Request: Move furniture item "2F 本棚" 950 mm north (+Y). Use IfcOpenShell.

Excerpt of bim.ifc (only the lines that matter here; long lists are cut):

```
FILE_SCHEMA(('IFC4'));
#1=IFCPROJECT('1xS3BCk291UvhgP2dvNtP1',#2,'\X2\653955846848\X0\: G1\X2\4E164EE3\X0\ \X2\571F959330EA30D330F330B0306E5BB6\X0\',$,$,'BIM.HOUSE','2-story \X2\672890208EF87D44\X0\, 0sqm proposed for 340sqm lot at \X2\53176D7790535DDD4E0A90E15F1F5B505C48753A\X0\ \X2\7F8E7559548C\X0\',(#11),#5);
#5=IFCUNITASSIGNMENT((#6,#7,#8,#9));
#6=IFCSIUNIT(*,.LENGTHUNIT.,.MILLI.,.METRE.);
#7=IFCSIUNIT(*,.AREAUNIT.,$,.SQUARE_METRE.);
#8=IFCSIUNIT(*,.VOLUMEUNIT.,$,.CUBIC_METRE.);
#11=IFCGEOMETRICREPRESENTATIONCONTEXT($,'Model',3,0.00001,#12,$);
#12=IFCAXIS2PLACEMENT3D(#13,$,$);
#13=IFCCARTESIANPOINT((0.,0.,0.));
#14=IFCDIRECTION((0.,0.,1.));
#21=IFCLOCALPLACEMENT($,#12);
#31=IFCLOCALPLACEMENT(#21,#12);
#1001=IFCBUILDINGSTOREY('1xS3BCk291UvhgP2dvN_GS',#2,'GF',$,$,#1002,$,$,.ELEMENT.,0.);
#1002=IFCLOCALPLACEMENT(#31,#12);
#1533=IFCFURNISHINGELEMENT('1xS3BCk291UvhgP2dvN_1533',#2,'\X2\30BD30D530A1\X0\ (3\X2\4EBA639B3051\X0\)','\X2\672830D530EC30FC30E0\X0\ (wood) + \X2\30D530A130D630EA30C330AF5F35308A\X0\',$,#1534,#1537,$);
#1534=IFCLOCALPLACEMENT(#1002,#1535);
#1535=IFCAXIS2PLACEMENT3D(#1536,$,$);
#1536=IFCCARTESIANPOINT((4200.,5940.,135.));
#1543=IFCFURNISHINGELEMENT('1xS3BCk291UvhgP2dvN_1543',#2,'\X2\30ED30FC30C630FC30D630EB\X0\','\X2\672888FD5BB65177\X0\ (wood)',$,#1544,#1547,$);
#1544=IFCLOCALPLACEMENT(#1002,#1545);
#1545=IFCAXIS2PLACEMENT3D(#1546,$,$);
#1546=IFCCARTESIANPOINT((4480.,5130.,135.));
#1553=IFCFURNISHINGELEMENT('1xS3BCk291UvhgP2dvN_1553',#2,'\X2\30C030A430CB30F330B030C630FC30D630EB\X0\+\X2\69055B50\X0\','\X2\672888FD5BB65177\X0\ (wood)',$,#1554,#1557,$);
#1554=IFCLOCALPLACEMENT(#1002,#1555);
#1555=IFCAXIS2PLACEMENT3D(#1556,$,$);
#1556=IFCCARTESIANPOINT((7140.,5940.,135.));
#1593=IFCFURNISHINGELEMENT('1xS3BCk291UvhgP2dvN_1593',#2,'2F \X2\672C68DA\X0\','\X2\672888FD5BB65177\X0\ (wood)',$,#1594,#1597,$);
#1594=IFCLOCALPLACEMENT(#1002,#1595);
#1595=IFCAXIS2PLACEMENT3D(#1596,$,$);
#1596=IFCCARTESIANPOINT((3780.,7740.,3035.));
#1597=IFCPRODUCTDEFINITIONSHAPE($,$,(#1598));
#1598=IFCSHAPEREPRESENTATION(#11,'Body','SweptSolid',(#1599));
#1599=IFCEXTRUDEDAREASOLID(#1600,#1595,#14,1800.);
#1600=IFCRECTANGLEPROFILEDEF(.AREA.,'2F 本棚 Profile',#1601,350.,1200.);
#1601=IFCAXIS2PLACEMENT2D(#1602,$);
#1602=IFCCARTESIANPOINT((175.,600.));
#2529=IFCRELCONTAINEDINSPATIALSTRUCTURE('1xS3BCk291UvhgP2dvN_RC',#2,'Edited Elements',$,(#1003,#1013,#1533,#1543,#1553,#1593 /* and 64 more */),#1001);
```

```python
import ifcopenshell
import ifcopenshell.api.geometry
import ifcopenshell.util.placement

model = ifcopenshell.open("bim.ifc")

item = model.by_guid("1xS3BCk291UvhgP2dvN_1593")
matrix = ifcopenshell.util.placement.get_local_placement(item.ObjectPlacement)
matrix[1, 3] += 950.0
ifcopenshell.api.geometry.edit_object_placement(model, product=item, matrix=matrix, is_si=False)

print(ifcopenshell.util.placement.get_local_placement(item.ObjectPlacement).round(3) + 0.0)

model.write("bim_v2.ifc")
```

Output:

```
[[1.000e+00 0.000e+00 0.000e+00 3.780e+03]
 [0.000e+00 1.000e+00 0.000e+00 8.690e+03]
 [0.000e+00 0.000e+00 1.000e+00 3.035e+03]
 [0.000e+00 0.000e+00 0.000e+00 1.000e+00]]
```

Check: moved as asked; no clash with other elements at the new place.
